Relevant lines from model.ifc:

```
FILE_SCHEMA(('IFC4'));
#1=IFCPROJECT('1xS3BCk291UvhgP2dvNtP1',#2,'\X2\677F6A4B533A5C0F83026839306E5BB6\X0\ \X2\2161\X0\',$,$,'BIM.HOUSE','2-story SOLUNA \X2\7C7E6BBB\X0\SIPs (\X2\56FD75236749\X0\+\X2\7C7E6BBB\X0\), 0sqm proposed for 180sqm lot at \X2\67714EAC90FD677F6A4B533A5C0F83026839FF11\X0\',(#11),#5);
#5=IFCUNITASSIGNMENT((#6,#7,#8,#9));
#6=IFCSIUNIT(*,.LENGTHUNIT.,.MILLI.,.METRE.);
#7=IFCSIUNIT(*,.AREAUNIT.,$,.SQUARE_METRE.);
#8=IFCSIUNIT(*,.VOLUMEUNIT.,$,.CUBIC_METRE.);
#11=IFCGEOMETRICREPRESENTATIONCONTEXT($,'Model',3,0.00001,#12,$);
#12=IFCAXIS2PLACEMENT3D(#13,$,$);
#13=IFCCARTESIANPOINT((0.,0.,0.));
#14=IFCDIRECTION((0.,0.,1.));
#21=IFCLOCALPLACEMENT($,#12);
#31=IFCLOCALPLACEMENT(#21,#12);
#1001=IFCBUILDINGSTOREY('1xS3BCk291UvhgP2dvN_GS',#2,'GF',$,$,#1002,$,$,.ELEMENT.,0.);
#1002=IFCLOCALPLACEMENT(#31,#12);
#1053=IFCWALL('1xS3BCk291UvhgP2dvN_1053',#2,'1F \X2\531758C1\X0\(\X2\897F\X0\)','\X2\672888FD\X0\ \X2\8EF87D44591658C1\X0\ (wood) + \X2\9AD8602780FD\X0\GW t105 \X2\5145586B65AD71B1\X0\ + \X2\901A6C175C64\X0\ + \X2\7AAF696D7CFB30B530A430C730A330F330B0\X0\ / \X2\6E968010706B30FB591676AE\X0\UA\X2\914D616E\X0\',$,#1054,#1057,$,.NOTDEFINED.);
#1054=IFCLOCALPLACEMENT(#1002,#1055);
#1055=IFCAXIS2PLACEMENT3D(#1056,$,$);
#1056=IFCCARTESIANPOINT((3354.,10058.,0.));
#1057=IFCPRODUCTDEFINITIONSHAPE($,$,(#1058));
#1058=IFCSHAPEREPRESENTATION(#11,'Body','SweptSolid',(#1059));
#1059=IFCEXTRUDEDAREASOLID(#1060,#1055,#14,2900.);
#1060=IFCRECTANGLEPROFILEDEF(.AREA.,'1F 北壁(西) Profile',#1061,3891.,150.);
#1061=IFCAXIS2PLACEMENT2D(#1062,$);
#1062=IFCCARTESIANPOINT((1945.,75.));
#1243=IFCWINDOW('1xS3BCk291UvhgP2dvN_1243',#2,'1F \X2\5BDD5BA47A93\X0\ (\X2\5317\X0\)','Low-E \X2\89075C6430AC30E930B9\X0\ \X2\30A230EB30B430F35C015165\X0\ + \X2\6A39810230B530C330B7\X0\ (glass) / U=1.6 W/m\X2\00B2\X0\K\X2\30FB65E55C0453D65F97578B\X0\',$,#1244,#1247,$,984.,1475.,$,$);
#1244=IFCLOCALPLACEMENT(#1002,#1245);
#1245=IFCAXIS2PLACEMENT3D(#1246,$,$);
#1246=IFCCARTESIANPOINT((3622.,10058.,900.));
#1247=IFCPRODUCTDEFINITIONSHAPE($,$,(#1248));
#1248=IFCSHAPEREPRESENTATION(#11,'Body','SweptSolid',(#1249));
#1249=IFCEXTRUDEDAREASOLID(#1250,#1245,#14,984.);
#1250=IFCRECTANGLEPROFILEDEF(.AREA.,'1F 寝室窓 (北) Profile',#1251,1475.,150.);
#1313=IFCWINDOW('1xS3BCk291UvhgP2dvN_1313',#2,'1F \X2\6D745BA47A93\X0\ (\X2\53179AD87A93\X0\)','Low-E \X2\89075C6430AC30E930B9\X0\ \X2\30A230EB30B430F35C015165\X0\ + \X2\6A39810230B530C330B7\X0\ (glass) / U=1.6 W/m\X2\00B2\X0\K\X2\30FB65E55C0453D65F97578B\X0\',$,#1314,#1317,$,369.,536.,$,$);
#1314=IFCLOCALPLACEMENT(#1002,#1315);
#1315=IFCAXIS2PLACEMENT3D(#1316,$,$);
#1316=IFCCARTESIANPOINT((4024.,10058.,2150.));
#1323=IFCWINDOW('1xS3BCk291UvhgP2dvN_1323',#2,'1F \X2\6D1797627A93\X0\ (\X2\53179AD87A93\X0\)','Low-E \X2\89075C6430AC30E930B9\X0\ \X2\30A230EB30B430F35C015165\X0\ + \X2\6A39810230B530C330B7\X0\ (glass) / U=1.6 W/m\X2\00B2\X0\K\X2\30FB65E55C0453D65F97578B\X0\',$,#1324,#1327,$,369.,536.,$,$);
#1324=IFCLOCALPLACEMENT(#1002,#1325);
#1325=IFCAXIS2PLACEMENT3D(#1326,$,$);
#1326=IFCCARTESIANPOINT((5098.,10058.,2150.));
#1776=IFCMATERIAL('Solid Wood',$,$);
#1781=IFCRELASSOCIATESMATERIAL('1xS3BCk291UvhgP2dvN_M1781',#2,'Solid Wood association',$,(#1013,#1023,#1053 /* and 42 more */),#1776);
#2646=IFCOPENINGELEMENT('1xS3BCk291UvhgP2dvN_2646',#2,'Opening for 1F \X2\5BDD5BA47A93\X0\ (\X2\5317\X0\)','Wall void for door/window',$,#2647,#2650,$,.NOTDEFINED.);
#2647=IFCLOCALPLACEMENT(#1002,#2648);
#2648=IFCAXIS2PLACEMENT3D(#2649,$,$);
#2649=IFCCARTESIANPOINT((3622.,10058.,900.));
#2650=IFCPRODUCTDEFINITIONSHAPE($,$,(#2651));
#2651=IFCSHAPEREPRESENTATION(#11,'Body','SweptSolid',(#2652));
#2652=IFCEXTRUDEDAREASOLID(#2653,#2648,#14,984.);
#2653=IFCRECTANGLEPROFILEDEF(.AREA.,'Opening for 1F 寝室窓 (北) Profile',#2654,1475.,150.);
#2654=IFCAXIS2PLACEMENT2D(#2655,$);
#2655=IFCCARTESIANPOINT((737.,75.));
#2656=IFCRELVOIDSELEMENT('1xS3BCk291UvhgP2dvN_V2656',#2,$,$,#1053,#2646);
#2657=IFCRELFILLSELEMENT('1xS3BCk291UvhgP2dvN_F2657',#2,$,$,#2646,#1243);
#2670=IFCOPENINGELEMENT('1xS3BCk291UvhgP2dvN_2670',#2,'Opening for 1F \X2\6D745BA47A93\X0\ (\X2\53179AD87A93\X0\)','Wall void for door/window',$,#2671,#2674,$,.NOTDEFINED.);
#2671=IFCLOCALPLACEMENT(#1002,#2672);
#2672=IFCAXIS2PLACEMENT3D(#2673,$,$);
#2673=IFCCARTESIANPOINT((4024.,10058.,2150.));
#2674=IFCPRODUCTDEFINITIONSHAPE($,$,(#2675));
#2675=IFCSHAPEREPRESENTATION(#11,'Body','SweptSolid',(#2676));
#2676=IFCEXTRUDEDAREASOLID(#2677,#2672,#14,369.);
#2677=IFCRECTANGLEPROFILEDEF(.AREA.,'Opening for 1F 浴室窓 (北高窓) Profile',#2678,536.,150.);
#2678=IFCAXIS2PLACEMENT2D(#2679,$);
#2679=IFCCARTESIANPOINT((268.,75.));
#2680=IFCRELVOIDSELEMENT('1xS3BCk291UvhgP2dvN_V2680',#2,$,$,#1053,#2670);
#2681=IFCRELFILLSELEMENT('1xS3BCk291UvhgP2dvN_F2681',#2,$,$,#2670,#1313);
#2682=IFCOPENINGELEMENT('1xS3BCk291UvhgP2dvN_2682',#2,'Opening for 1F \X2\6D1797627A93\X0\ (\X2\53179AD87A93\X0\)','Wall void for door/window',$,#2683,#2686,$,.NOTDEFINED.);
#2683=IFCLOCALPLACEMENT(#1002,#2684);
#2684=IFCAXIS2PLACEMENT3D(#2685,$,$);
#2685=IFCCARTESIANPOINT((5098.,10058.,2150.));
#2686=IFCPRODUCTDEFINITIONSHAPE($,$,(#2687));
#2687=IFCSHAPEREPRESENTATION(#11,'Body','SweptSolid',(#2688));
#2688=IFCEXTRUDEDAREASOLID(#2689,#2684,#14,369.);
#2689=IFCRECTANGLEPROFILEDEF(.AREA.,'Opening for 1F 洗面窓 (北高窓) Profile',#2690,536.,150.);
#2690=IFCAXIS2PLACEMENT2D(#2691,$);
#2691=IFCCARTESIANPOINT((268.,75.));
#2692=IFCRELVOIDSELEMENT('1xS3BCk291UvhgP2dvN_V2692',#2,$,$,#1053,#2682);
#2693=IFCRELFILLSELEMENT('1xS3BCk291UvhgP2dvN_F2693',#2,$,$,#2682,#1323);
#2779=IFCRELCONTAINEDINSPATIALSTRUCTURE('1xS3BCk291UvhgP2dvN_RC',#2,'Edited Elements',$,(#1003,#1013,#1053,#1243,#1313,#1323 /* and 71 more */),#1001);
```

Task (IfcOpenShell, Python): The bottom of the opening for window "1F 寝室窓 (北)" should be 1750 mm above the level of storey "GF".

```python
import numpy as np
import ifcopenshell
import ifcopenshell.api.geometry
import ifcopenshell.geom
import ifcopenshell.util.element
import ifcopenshell.util.placement
import ifcopenshell.util.shape
import ifcopenshell.util.unit

model = ifcopenshell.open("model.ifc")
unit_scale = ifcopenshell.util.unit.calculate_unit_scale(model)

window = model.by_id(1243)
opening = window.FillsVoids[0].RelatingOpeningElement
storey = ifcopenshell.util.element.get_container(window, ifc_class="IfcBuildingStorey")
level = ifcopenshell.util.placement.get_local_placement(storey.ObjectPlacement)[2, 3]

# The opening's origin need not be at the sill, so measure its lowest point.
shape = ifcopenshell.geom.create_shape(ifcopenshell.geom.settings(), opening)
bottom = ifcopenshell.util.shape.get_shape_bottom_elevation(shape, shape.geometry) / unit_scale
dz = level + 1.75 / unit_scale - bottom

shift = np.array([0.0, 0.0, dz])
# The window is not placed relative to its opening, so move both.
for product in (opening, window):
    matrix = ifcopenshell.util.placement.get_local_placement(product.ObjectPlacement)
    matrix[:3, 3] += shift
    ifcopenshell.api.geometry.edit_object_placement(model, product=product, matrix=matrix, is_si=False)

print(f"moved by {dz * unit_scale:+.3f} m")

model.write("model_v2.ifc")
```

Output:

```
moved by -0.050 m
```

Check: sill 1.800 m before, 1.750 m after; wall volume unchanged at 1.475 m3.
